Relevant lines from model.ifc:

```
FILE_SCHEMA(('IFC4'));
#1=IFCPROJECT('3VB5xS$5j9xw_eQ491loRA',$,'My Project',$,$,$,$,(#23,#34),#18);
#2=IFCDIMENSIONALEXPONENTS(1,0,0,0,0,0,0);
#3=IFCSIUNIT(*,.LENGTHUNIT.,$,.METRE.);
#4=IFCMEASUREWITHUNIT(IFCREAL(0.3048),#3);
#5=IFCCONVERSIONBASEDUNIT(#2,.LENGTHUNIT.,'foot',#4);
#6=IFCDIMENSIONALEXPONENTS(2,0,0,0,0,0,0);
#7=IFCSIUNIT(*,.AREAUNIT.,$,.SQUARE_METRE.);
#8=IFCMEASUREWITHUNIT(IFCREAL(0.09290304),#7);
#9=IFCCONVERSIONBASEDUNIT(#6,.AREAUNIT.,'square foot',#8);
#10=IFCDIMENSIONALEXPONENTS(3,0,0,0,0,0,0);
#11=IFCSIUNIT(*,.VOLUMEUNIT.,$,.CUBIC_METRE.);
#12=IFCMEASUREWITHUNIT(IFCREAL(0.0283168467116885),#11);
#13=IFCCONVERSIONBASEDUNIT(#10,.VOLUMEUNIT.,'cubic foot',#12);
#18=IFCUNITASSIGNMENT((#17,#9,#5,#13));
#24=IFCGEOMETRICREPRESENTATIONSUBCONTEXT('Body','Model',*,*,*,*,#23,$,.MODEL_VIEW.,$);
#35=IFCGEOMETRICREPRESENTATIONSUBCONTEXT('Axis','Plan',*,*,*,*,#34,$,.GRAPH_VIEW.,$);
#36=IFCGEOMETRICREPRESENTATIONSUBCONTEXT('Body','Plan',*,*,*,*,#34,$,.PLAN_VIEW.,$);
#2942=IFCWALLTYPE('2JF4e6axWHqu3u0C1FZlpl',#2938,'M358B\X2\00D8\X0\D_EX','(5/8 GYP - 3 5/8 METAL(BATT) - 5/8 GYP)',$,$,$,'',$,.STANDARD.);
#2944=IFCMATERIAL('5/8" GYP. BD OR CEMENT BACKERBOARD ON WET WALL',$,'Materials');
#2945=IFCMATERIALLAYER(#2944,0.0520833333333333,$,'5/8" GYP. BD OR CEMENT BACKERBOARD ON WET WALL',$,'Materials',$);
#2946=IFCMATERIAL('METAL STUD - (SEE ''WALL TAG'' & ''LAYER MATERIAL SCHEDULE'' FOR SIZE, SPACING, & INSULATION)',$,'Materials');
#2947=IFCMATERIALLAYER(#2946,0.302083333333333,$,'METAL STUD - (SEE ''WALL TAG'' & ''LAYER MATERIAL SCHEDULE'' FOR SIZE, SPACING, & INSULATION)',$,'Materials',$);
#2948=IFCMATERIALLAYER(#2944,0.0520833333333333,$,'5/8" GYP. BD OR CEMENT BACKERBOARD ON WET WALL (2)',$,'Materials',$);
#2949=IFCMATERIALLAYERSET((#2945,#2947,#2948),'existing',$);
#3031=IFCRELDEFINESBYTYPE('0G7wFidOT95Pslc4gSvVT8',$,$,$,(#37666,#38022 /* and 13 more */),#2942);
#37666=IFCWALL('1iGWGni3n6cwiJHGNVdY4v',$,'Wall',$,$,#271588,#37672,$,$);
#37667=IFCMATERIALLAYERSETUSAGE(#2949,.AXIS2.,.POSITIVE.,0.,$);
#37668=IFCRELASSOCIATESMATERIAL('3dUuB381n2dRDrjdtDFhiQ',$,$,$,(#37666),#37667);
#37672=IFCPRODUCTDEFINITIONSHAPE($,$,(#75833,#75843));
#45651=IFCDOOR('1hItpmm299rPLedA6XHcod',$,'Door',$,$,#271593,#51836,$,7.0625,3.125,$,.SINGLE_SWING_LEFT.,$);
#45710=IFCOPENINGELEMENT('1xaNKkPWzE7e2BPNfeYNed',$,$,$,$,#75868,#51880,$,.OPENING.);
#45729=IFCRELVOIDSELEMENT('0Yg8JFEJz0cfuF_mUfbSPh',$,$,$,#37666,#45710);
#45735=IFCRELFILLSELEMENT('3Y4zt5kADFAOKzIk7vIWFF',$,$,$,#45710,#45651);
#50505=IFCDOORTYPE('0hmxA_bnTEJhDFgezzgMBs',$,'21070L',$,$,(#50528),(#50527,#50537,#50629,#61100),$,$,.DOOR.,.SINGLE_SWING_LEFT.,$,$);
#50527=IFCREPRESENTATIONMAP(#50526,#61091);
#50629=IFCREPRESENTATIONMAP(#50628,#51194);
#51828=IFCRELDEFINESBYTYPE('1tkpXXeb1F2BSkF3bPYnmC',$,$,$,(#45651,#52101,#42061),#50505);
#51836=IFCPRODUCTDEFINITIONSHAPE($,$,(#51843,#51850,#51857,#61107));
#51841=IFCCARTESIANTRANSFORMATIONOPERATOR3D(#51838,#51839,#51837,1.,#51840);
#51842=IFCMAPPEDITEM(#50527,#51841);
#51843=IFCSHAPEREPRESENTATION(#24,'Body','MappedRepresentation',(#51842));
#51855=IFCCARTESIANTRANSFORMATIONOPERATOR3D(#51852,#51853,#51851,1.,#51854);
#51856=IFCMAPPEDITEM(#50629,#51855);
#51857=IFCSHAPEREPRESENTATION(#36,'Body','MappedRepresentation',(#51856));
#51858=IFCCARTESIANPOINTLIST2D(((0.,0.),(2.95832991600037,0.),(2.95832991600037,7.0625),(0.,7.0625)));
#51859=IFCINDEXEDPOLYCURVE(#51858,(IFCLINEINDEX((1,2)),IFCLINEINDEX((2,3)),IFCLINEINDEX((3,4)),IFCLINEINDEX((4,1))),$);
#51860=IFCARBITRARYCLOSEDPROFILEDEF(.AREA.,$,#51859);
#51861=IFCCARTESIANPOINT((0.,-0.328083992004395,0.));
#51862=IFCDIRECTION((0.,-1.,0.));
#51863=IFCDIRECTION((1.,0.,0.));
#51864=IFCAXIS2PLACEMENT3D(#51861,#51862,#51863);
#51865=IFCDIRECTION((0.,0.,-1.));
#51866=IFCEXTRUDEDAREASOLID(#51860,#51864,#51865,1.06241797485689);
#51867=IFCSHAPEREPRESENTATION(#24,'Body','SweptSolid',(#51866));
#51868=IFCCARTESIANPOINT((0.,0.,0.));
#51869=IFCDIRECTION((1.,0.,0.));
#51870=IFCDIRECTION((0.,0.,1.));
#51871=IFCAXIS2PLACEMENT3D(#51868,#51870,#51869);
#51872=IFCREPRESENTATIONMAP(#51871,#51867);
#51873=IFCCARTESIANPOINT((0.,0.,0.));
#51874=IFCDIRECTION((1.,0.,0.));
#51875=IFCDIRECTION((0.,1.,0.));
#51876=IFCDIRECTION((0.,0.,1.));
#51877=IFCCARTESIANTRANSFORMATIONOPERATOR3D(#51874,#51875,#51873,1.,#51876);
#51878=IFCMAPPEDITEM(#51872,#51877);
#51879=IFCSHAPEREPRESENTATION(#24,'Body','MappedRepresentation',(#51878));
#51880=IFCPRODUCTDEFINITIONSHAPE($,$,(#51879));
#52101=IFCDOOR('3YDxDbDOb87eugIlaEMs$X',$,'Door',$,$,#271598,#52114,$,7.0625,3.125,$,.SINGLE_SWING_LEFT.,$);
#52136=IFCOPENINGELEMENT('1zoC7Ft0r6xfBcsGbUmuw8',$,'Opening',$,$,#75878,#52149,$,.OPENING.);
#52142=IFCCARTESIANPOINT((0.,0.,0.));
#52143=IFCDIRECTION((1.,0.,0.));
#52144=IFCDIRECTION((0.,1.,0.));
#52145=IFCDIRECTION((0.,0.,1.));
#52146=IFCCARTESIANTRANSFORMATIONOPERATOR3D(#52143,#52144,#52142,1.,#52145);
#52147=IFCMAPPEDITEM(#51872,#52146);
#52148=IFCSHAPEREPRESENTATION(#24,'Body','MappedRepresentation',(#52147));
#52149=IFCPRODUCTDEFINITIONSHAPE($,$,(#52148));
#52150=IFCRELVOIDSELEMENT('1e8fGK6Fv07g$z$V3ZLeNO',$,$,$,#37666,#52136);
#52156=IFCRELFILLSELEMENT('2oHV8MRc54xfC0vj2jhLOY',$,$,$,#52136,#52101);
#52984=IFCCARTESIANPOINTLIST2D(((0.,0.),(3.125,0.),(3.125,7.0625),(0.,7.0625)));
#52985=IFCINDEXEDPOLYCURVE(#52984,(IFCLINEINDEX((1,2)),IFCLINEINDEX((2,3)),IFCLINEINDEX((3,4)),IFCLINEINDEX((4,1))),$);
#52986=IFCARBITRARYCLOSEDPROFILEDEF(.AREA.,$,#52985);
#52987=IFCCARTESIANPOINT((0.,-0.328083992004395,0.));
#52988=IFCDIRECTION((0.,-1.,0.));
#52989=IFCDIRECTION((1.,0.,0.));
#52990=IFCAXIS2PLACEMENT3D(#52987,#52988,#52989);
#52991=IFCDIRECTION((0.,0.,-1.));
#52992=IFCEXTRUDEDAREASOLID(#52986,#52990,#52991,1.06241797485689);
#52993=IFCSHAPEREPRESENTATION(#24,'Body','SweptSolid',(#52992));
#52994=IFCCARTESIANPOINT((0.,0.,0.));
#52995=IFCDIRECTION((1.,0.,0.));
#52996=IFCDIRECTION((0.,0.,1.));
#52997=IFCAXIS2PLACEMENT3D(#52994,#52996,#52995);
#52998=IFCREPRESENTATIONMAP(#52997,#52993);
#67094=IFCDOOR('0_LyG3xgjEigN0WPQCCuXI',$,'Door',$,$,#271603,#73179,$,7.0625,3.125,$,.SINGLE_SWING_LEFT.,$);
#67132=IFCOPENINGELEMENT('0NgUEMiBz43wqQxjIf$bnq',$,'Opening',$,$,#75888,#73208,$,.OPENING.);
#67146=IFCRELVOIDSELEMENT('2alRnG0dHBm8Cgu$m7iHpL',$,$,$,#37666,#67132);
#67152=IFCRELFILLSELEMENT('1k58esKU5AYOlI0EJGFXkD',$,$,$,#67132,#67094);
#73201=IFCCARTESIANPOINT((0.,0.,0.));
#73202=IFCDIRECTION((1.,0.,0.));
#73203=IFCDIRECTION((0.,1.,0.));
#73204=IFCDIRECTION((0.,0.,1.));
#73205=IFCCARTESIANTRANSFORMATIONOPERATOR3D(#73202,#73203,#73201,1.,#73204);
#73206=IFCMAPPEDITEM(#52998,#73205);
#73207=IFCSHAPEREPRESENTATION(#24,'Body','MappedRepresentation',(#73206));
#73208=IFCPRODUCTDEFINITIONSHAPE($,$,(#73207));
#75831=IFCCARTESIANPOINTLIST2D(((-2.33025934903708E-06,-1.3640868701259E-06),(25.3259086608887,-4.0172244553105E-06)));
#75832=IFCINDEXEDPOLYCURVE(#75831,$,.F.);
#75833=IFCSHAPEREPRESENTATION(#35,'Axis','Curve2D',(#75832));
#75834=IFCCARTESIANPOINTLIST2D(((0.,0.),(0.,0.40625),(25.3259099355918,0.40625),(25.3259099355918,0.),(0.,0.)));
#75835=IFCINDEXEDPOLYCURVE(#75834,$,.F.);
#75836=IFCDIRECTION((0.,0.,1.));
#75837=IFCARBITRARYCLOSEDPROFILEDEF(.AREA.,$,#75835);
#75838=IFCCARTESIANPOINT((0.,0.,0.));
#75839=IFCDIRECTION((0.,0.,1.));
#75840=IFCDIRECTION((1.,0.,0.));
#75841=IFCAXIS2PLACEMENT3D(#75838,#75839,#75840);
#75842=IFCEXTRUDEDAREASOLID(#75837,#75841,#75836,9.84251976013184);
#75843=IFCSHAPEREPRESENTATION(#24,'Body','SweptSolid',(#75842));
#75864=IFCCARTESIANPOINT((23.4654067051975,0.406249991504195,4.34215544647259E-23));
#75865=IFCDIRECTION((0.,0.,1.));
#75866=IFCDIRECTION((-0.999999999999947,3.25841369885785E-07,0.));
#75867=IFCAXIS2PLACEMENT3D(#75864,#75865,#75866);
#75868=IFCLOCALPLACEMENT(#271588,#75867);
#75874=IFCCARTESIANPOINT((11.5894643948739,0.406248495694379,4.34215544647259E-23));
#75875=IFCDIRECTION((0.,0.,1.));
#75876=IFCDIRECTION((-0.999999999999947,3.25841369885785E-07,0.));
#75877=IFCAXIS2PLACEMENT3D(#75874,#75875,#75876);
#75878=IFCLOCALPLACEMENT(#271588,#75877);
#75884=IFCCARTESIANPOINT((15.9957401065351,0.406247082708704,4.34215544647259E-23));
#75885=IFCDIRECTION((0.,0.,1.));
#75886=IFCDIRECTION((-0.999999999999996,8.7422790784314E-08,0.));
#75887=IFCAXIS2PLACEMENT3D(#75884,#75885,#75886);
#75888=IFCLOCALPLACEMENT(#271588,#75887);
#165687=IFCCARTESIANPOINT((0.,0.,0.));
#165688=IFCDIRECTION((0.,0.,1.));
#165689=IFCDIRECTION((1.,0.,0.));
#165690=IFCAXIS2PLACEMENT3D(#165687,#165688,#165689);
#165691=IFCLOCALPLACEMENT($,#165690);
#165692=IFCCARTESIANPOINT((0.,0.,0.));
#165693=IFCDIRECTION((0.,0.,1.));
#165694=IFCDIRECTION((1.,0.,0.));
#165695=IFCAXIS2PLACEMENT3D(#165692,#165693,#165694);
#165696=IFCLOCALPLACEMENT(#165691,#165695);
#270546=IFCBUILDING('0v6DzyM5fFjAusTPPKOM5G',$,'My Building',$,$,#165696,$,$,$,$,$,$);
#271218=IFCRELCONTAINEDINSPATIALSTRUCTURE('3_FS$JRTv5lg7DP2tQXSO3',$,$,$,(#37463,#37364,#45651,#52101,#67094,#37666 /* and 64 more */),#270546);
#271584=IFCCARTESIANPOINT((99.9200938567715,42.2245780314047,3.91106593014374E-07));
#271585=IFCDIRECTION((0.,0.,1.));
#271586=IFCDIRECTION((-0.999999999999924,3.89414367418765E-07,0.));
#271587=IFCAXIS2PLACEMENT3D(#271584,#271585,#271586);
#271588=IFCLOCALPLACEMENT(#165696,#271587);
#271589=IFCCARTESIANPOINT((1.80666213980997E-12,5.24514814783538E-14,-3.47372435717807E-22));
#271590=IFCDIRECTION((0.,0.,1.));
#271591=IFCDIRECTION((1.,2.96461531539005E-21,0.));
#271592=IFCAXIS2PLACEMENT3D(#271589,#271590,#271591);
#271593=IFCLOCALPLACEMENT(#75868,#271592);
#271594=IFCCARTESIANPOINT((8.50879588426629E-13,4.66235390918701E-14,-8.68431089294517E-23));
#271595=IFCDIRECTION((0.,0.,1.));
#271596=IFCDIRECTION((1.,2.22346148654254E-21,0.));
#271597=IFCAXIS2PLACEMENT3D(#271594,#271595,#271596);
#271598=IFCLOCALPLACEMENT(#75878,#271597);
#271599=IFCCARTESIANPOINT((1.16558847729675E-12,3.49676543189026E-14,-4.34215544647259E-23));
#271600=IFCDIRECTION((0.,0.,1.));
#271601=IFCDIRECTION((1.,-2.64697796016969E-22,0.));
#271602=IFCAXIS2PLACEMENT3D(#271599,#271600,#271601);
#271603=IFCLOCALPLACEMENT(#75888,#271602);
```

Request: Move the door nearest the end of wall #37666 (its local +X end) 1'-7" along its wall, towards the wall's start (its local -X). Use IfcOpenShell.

```python
import ifcopenshell
import ifcopenshell.api.geometry
import ifcopenshell.util.placement
import ifcopenshell.util.unit

model = ifcopenshell.open("model.ifc")
unit_scale = ifcopenshell.util.unit.calculate_unit_scale(model)

door = model.by_id(45651)
opening = door.FillsVoids[0].RelatingOpeningElement
wall = opening.VoidsElements[0].RelatingBuildingElement

wall_matrix = ifcopenshell.util.placement.get_local_placement(wall.ObjectPlacement)
shift = wall_matrix[:3, 0] * -19 * 0.0254 / unit_scale
before = ifcopenshell.util.placement.get_local_placement(door.ObjectPlacement)[:3, 3].copy()

# The door is placed relative to its opening, so it follows when the opening moves.
matrix = ifcopenshell.util.placement.get_local_placement(opening.ObjectPlacement)
matrix[:3, 3] += shift
ifcopenshell.api.geometry.edit_object_placement(
    model, product=opening, matrix=matrix, is_si=False, should_transform_children=True
)

after = ifcopenshell.util.placement.get_local_placement(door.ObjectPlacement)[:3, 3]
print("door moved by", (after - before).round(3) + 0.0)

model.write("model_updated.ifc")
```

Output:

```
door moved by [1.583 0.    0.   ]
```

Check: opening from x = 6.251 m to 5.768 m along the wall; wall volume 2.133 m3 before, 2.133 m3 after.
